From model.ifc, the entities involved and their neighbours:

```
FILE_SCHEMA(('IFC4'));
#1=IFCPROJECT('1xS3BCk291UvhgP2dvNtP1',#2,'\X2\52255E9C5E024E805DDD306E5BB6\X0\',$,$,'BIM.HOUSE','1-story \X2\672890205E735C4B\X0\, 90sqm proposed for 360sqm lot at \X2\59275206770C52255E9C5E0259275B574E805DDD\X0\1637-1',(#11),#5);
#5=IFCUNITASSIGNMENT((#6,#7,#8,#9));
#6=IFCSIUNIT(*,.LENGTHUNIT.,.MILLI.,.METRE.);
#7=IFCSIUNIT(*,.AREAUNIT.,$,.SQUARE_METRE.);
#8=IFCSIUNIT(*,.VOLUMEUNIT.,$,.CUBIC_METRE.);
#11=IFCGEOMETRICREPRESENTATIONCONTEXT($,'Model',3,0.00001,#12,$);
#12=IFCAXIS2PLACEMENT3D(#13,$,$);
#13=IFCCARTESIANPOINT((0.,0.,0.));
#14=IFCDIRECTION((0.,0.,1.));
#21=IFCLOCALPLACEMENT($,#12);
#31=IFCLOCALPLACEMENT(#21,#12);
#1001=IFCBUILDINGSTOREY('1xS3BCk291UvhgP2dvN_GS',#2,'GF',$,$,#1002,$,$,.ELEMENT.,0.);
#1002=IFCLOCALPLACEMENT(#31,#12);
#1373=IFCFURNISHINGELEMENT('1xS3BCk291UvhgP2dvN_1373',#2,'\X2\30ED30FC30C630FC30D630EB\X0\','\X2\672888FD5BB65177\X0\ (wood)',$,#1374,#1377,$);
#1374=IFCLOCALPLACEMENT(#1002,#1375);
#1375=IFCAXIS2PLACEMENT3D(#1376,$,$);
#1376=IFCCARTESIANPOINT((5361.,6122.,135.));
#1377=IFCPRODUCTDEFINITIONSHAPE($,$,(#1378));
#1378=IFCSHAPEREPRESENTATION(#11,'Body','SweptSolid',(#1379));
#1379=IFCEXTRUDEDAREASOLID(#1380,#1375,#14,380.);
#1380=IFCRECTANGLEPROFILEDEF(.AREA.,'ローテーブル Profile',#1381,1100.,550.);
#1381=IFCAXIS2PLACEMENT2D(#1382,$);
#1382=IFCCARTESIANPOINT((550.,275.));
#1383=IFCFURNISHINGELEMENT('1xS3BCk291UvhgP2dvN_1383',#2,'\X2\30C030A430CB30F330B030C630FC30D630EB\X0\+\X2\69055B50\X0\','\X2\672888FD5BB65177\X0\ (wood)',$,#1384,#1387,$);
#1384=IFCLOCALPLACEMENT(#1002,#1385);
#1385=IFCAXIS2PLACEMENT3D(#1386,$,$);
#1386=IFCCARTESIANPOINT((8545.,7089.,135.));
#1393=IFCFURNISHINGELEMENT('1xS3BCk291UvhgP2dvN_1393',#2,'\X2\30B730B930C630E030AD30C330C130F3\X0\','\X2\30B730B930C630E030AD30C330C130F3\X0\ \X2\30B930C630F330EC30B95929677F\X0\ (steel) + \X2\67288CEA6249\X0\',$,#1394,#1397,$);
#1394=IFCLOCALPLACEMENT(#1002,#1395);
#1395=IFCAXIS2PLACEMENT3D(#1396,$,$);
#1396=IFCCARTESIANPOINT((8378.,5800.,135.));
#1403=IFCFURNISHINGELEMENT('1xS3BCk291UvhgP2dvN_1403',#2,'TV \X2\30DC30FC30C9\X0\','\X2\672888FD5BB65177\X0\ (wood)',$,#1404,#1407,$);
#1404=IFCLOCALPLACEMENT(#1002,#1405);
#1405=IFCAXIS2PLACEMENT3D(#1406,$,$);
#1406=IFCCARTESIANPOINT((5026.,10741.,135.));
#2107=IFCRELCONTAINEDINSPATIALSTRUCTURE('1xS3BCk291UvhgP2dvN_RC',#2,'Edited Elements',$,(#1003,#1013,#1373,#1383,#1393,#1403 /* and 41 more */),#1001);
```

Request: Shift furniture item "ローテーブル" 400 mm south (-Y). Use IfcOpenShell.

```python
import ifcopenshell
import ifcopenshell.api.geometry
import ifcopenshell.util.placement
import ifcopenshell.util.unit

model = ifcopenshell.open("model.ifc")
unit_scale = ifcopenshell.util.unit.calculate_unit_scale(model)

item = model.by_guid("1xS3BCk291UvhgP2dvN_1373")
matrix = ifcopenshell.util.placement.get_local_placement(item.ObjectPlacement)
matrix[1, 3] -= 0.4 / unit_scale
ifcopenshell.api.geometry.edit_object_placement(model, product=item, matrix=matrix, is_si=False)

print(ifcopenshell.util.placement.get_local_placement(item.ObjectPlacement).round(3) + 0.0)

model.write("model_updated.ifc")
```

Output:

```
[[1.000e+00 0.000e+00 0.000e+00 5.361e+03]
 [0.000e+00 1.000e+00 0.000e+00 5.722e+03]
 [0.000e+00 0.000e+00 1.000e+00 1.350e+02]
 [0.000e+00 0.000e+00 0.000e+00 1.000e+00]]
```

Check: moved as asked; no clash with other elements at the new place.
